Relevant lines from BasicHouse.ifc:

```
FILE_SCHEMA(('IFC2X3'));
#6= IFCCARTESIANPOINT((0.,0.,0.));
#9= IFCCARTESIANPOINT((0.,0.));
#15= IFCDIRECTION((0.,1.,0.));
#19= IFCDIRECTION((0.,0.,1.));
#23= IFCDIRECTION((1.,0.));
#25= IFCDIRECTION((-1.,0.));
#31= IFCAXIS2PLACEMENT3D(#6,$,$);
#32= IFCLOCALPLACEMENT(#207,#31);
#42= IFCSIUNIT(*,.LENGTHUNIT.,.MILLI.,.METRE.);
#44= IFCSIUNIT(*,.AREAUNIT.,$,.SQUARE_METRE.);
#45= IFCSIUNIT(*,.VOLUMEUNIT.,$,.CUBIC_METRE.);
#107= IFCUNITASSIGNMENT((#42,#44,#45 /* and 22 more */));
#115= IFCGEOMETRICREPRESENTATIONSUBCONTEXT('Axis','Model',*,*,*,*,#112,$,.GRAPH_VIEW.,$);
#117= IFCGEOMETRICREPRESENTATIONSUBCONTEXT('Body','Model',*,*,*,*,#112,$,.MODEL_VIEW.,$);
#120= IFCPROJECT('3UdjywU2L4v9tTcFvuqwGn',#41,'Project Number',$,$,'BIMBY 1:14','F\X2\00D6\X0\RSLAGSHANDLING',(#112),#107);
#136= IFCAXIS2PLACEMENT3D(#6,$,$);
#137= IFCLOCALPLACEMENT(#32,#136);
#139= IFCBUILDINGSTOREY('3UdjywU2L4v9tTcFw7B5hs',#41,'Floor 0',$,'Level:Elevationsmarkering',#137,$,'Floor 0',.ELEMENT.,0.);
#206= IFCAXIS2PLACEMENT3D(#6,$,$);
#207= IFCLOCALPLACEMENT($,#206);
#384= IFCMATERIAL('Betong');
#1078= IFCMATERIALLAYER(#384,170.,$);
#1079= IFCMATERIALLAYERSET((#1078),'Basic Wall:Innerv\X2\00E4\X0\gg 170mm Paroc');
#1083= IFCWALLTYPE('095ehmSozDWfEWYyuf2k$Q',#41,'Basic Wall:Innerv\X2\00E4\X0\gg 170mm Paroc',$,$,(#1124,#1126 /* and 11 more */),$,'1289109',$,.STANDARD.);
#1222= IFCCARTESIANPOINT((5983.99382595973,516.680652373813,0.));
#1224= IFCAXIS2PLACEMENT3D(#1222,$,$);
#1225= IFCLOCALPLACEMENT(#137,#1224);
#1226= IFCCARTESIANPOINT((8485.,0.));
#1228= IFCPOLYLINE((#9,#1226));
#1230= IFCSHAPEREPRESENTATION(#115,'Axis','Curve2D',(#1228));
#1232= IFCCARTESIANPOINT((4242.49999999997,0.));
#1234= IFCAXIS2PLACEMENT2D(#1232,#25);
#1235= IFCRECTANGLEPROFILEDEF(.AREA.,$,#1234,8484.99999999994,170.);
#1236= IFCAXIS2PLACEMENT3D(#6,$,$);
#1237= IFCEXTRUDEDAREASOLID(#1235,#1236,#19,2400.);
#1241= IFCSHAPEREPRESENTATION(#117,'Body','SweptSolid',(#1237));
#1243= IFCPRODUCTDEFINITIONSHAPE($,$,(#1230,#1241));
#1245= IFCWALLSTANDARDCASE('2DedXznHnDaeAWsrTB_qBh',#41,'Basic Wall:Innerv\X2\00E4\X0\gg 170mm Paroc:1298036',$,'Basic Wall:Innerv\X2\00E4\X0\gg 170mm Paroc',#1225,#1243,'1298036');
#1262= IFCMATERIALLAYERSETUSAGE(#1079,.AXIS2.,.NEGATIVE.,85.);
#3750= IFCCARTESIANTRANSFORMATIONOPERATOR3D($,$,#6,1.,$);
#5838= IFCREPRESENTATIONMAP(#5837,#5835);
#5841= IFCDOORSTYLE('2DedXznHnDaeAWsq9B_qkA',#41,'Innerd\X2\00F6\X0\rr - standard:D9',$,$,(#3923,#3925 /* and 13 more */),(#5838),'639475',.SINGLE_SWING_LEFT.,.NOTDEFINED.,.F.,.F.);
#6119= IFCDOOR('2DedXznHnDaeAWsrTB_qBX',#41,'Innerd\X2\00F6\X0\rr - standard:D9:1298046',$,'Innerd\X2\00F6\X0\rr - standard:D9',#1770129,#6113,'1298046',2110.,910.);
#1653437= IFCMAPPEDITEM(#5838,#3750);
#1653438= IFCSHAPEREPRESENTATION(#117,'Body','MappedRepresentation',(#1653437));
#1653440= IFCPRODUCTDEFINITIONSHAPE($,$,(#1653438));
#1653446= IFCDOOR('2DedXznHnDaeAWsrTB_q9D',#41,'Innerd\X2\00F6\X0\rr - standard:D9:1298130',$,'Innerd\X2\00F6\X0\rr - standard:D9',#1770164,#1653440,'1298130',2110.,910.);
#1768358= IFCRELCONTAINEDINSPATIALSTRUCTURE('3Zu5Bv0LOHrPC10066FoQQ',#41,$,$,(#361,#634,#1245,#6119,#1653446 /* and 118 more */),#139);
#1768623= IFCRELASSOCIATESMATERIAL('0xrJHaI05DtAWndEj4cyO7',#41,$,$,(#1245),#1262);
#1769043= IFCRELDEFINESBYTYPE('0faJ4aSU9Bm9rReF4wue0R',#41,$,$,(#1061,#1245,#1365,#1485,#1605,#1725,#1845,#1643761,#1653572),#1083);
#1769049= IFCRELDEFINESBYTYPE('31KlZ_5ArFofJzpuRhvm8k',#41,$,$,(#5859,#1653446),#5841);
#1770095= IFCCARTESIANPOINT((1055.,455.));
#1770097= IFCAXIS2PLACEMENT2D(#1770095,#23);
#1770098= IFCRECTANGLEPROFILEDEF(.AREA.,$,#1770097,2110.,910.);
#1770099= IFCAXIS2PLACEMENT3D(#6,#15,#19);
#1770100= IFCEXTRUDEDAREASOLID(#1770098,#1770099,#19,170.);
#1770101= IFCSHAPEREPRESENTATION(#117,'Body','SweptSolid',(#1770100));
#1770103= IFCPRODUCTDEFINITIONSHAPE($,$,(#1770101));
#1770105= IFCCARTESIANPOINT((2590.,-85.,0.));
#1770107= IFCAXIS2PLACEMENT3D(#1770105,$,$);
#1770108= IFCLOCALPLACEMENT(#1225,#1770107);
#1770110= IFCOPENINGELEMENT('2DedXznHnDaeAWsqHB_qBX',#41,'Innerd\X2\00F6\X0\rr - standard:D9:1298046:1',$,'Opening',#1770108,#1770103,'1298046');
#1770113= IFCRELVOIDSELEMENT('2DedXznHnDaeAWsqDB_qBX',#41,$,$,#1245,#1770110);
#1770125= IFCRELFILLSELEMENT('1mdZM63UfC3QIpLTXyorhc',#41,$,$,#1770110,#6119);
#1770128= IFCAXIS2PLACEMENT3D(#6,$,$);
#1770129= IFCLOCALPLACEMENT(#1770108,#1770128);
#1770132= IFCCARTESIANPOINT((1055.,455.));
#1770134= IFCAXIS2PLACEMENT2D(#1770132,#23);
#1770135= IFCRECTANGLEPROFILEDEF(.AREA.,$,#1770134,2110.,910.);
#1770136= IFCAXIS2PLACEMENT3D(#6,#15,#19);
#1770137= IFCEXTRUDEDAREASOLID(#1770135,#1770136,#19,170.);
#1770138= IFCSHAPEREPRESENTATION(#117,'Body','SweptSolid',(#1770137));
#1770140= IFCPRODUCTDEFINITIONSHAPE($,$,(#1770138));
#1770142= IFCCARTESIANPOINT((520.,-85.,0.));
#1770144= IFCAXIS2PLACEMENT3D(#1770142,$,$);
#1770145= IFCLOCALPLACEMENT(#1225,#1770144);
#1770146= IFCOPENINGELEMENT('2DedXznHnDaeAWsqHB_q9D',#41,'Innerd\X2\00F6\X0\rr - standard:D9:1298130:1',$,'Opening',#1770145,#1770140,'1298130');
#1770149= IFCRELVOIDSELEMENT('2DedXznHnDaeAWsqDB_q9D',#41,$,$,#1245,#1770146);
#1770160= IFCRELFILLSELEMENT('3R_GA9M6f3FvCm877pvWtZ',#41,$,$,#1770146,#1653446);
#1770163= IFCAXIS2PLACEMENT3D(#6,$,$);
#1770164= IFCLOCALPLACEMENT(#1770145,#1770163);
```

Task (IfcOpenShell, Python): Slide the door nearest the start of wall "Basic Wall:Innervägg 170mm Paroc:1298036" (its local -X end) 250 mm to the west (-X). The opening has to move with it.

```python
import ifcopenshell
import ifcopenshell.api.geometry
import ifcopenshell.util.placement
import ifcopenshell.util.unit

model = ifcopenshell.open("BasicHouse.ifc")
unit_scale = ifcopenshell.util.unit.calculate_unit_scale(model)

door = model.by_id(1653446)
opening = door.FillsVoids[0].RelatingOpeningElement
wall = opening.VoidsElements[0].RelatingBuildingElement

wall_matrix = ifcopenshell.util.placement.get_local_placement(wall.ObjectPlacement)
shift = wall_matrix[:3, 0] * -0.25 / unit_scale
before = ifcopenshell.util.placement.get_local_placement(door.ObjectPlacement)[:3, 3].copy()

# The door is placed relative to its opening, so it follows when the opening moves.
matrix = ifcopenshell.util.placement.get_local_placement(opening.ObjectPlacement)
matrix[:3, 3] += shift
ifcopenshell.api.geometry.edit_object_placement(
    model, product=opening, matrix=matrix, is_si=False, should_transform_children=True
)

after = ifcopenshell.util.placement.get_local_placement(door.ObjectPlacement)[:3, 3]
print("door moved by", (after - before).round(3) + 0.0)

model.write("BasicHouse_edited.ifc")
```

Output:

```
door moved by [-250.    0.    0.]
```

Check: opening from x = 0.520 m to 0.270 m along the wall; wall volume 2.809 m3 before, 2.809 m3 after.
